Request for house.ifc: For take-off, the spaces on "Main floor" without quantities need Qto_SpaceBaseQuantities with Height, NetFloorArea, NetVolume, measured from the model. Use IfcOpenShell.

First a look at what the model holds.

```python
import ifcopenshell
import ifcopenshell.util.element
import ifcopenshell.util.unit

model = ifcopenshell.open("house.ifc")
print(model.schema)
for unit_type in ("LENGTHUNIT", "AREAUNIT", "VOLUMEUNIT"):
    print(unit_type, ifcopenshell.util.unit.calculate_unit_scale(model, unit_type))
storey = next(s for s in model.by_type("IfcBuildingStorey") if s.Name == "Main floor")
spaces = [e for e in ifcopenshell.util.element.get_decomposition(storey) if e.is_a("IfcSpace")]
for e in sorted(spaces, key=lambda e: e.id()):
    print(e.id(), e.is_a(), e.Name, list(ifcopenshell.util.element.get_psets(e, qtos_only=True)), sep=" | ")
```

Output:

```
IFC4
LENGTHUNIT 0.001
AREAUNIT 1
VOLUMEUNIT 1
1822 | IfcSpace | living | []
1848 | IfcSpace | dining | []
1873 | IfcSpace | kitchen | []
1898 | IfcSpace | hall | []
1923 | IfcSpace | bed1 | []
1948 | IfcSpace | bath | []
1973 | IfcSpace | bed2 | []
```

```python
import ifcopenshell
import ifcopenshell.api.pset
import ifcopenshell.geom
import ifcopenshell.util.element
import ifcopenshell.util.shape
import ifcopenshell.util.unit

model = ifcopenshell.open("house.ifc")
unit_scale = ifcopenshell.util.unit.calculate_unit_scale(model)
area_scale = ifcopenshell.util.unit.calculate_unit_scale(model, "AREAUNIT")
volume_scale = ifcopenshell.util.unit.calculate_unit_scale(model, "VOLUMEUNIT")
settings = ifcopenshell.geom.settings()

storey = next(s for s in model.by_type("IfcBuildingStorey") if s.Name == "Main floor")
spaces = [e for e in ifcopenshell.util.element.get_decomposition(storey) if e.is_a("IfcSpace")]

for e in sorted(spaces, key=lambda e: e.id()):
    if ifcopenshell.util.element.get_psets(e, qtos_only=True, should_inherit=False):
        continue
    # Geometry comes back in metres, in the element's own axes.
    shape = ifcopenshell.geom.create_shape(settings, e)
    values = {
        "Height": ifcopenshell.util.shape.get_z(shape.geometry) / unit_scale,
        "NetFloorArea": ifcopenshell.util.shape.get_footprint_area(shape.geometry) / area_scale,
        "NetVolume": ifcopenshell.util.shape.get_volume(shape.geometry) / volume_scale,
    }
    qto = ifcopenshell.api.pset.add_qto(model, product=e, name="Qto_SpaceBaseQuantities")
    ifcopenshell.api.pset.edit_qto(model, qto=qto, properties=values)
    print(e.id(), {k: round(v, 3) for k, v in values.items()})

model.write("house_v2.ifc")
```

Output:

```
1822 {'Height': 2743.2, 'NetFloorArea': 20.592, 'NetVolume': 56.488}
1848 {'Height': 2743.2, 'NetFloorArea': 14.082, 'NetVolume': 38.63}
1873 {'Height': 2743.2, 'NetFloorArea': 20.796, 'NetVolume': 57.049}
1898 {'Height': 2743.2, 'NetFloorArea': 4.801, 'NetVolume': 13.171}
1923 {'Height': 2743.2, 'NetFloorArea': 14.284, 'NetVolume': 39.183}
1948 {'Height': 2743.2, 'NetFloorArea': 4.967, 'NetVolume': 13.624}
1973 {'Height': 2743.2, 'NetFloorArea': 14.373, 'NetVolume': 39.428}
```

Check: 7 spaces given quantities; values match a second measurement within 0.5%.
